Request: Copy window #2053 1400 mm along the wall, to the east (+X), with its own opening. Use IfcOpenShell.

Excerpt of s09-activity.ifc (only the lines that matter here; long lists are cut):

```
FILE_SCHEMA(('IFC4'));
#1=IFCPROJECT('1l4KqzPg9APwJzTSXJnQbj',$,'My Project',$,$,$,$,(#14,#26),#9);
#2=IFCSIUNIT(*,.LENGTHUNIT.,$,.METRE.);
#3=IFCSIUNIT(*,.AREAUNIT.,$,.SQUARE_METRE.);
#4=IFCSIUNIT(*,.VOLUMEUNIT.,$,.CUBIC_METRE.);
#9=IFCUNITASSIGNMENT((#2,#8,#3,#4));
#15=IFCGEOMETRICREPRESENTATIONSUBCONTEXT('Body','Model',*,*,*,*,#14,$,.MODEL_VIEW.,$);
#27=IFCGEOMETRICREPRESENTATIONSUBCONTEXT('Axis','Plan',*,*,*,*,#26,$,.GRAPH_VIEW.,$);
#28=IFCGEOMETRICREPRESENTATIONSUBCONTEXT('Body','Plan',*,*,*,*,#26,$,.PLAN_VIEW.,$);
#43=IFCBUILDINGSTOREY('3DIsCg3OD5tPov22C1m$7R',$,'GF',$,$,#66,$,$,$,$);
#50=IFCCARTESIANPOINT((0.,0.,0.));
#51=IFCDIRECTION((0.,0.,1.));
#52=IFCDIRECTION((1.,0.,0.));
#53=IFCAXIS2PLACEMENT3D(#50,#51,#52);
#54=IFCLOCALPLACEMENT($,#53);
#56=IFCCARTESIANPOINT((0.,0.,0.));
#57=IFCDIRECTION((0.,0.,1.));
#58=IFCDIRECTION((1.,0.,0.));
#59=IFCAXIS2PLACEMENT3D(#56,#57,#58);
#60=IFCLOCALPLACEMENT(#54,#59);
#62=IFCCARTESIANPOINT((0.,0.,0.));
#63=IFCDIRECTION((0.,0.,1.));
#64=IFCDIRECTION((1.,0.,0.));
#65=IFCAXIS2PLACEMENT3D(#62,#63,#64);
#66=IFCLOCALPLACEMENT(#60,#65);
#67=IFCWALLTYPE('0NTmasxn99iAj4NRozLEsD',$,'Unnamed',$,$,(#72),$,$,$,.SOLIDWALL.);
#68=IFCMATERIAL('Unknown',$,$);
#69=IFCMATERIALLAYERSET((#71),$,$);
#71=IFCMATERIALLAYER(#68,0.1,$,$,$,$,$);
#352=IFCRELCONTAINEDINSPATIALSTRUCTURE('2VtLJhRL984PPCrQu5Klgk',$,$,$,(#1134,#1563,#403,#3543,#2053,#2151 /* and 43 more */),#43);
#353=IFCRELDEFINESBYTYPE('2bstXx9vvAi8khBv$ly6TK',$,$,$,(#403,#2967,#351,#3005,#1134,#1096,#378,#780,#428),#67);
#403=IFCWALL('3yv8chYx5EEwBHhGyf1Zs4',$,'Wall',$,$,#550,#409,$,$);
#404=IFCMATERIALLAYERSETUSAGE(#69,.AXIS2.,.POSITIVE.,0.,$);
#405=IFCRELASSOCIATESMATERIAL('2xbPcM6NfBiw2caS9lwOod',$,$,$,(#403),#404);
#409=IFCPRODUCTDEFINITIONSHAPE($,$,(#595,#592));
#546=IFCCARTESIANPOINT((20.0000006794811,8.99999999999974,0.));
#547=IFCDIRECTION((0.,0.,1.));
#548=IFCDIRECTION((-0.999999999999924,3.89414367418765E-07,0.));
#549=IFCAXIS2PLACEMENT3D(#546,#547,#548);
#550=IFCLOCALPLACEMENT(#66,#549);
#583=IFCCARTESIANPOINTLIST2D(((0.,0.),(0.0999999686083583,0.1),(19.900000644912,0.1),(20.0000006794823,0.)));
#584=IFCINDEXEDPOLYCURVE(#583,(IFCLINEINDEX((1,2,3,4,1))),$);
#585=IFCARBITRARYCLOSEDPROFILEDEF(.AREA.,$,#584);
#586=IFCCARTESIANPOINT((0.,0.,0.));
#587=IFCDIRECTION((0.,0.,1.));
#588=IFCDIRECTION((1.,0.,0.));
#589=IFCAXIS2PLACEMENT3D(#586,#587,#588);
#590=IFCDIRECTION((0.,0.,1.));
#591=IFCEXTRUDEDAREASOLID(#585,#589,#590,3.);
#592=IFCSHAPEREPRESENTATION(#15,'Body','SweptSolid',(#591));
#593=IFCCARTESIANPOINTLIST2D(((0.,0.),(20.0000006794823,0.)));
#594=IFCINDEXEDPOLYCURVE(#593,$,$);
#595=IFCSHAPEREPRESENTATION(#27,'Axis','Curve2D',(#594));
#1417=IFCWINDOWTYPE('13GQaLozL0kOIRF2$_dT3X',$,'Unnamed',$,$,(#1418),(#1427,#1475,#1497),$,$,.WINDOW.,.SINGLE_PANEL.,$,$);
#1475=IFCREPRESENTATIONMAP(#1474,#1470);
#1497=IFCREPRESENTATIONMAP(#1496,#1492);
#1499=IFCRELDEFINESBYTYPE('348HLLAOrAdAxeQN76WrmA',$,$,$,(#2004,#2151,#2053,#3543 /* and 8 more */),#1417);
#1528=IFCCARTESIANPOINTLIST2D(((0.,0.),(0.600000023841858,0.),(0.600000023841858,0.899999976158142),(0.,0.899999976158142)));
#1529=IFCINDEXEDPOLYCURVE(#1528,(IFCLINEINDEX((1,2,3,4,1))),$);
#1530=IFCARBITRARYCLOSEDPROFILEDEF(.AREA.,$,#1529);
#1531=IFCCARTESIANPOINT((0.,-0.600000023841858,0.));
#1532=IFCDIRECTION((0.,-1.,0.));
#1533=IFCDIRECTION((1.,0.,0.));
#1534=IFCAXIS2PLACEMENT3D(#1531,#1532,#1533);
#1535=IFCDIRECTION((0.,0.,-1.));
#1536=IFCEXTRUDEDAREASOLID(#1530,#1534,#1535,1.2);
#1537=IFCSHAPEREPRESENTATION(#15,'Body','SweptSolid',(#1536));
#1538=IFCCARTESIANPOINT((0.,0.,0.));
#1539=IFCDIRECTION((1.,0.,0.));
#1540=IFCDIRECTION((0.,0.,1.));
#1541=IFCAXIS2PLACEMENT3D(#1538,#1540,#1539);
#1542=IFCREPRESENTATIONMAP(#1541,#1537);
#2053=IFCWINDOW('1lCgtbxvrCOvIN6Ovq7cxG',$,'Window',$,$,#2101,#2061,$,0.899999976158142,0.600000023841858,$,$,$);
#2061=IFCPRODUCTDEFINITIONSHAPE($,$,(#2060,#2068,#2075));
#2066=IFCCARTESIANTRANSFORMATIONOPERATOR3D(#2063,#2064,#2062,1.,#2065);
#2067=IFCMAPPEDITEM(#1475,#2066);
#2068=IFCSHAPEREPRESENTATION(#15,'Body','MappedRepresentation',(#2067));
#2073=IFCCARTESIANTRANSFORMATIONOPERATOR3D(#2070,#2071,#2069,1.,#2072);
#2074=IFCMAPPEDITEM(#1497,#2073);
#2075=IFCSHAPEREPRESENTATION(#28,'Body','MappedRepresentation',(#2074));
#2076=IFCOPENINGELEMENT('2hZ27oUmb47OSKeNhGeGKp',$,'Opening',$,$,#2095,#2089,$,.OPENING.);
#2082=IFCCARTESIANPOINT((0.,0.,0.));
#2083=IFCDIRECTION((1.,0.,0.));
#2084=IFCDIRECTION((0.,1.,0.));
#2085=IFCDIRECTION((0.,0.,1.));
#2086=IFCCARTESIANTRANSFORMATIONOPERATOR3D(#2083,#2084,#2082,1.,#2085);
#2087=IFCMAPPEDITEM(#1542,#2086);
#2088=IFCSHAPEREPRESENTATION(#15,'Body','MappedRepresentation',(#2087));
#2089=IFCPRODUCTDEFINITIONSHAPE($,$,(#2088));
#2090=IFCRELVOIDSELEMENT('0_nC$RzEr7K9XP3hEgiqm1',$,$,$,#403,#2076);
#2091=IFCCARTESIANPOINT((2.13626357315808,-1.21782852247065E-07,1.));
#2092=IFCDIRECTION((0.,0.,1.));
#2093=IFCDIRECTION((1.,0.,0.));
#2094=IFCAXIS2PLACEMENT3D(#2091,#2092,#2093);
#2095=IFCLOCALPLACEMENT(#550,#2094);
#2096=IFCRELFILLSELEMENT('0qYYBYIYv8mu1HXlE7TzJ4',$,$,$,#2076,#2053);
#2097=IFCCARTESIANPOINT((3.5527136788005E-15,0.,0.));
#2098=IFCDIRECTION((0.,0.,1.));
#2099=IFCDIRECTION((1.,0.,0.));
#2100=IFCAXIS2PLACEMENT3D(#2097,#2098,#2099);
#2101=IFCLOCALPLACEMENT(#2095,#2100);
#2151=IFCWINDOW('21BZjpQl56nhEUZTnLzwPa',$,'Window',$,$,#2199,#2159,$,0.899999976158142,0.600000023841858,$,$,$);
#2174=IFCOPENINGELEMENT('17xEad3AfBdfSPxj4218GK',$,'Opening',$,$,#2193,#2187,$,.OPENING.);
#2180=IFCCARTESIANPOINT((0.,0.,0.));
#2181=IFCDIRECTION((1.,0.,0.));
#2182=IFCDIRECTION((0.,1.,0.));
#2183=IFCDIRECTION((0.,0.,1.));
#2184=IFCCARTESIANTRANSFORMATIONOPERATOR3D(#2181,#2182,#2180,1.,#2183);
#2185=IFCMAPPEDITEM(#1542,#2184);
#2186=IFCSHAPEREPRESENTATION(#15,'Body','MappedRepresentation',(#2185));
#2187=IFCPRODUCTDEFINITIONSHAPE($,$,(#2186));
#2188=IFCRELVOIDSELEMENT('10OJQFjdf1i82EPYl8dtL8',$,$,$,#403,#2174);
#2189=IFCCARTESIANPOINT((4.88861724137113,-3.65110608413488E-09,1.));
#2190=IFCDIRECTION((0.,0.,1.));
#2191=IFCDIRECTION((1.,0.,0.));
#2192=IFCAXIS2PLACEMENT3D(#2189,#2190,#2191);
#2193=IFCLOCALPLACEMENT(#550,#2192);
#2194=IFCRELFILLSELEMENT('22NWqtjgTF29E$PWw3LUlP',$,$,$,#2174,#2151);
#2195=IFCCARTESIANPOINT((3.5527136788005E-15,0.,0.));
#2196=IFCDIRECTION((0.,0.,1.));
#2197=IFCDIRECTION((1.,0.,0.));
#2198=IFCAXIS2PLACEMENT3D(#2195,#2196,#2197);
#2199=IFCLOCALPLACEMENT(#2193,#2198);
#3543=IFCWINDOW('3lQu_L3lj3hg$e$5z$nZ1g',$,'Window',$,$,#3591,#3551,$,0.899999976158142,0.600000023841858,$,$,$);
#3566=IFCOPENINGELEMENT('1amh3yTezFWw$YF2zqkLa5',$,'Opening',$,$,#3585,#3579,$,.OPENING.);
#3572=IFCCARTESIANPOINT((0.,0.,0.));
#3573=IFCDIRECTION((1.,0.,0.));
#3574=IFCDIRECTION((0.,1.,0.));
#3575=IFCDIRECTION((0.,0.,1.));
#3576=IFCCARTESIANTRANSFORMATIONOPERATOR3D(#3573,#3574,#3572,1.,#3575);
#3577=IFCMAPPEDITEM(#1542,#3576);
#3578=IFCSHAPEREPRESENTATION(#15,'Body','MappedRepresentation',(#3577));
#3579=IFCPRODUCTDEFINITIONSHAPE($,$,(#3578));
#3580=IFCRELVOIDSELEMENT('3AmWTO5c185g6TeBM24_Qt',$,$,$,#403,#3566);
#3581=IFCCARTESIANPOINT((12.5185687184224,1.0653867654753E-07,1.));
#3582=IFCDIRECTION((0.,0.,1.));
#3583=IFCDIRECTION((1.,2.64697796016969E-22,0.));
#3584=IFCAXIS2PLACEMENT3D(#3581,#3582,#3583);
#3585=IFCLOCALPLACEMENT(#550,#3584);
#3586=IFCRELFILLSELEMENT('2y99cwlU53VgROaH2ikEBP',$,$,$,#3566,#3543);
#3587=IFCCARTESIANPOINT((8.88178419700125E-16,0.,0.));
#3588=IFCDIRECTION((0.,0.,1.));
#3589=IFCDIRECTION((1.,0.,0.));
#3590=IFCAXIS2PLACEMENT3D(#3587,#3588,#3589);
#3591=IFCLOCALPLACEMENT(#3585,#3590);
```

```python
import ifcopenshell
import ifcopenshell.api.feature
import ifcopenshell.api.geometry
import ifcopenshell.api.root
import ifcopenshell.geom
import ifcopenshell.util.element
import ifcopenshell.util.placement
import ifcopenshell.util.shape
import ifcopenshell.util.unit

model = ifcopenshell.open("s09-activity.ifc")
unit_scale = ifcopenshell.util.unit.calculate_unit_scale(model)
settings = ifcopenshell.geom.settings()


def volume(element):
    """Net volume in cubic metres, openings subtracted."""
    shape = ifcopenshell.geom.create_shape(settings, element)
    return ifcopenshell.util.shape.get_volume(shape.geometry)


window = model.by_guid("1lCgtbxvrCOvIN6Ovq7cxG")
opening = window.FillsVoids[0].RelatingOpeningElement
wall = opening.VoidsElements[0].RelatingBuildingElement
before = volume(wall)
shift = ifcopenshell.util.placement.get_local_placement(wall.ObjectPlacement)[:3, 0] * -1.4 / unit_scale

# copy_class copies the void relationship, type, container and properties, but no geometry.
new_opening = ifcopenshell.api.root.copy_class(model, product=opening)
new_opening.Representation = ifcopenshell.util.element.copy_deep(
    model, opening.Representation, exclude=["IfcGeometricRepresentationContext", "IfcRepresentationMap"]
)
new_window = ifcopenshell.api.root.copy_class(model, product=window)
new_window.Representation = ifcopenshell.util.element.copy_deep(
    model, window.Representation, exclude=["IfcGeometricRepresentationContext", "IfcRepresentationMap"]
)
ifcopenshell.api.feature.add_filling(model, opening=new_opening, element=new_window)

for old, new in ((opening, new_opening), (window, new_window)):
    matrix = ifcopenshell.util.placement.get_local_placement(old.ObjectPlacement)
    matrix[:3, 3] += shift
    ifcopenshell.api.geometry.edit_object_placement(model, product=new, matrix=matrix, is_si=False)

after = volume(wall)

print(f"wall volume {before:.3f} -> {after:.3f} m3")

model.write("s09-activity_v2.ifc")
```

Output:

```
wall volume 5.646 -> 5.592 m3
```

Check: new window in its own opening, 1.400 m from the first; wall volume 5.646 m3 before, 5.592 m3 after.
